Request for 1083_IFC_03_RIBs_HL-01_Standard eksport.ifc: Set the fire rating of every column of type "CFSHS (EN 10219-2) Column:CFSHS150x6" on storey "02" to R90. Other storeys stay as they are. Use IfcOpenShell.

First a look at what the model holds.

```python
import ifcopenshell
import ifcopenshell.util.element

model = ifcopenshell.open("1083_IFC_03_RIBs_HL-01_Standard eksport.ifc")
print(model.schema)
storey = next(s for s in model.by_type("IfcBuildingStorey") if s.Name == "02")
columns = [e for e in ifcopenshell.util.element.get_decomposition(storey) if e.is_a("IfcColumn")]
seen = {}
for e in columns:
    element_type = ifcopenshell.util.element.get_type(e)
    key = (element_type.Name if element_type != e and element_type else None, ifcopenshell.util.element.get_pset(e, "Pset_ColumnCommon", "FireRating"))
    seen[key] = seen.get(key, 0) + 1
for (name, value), count in sorted(seen.items(), key=str):
    print(count, "x", name, "|", value)
```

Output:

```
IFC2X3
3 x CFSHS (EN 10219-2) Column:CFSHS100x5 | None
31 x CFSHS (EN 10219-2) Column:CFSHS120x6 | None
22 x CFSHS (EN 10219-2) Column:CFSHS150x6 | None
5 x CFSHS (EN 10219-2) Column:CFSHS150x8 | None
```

```python
import ifcopenshell
import ifcopenshell.api.pset
import ifcopenshell.util.element

model = ifcopenshell.open("1083_IFC_03_RIBs_HL-01_Standard eksport.ifc")

storey = next(s for s in model.by_type("IfcBuildingStorey") if s.Name == "02")
columns = [e for e in ifcopenshell.util.element.get_decomposition(storey) if e.is_a("IfcColumn")]

count = 0
for e in columns:
    element_type = ifcopenshell.util.element.get_type(e)
    if element_type in (None, e) or element_type.Name != "CFSHS (EN 10219-2) Column:CFSHS150x6":
        continue
    # add_pset returns the element's existing set when there is one.
    pset = ifcopenshell.api.pset.add_pset(model, product=e, name="Pset_ColumnCommon")
    ifcopenshell.api.pset.edit_pset(model, pset=pset, properties={"FireRating": "R90"})
    count += 1

print(count, "columns updated")

model.write("1083_IFC_03_RIBs_HL-01_Standard eksport_updated.ifc")
```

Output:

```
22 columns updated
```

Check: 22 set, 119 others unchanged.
